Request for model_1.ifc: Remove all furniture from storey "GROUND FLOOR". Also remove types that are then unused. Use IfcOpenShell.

First a look at what the model holds.

```python
import ifcopenshell
import ifcopenshell.util.element

model = ifcopenshell.open("model_1.ifc")
print(model.schema)
storey = next(s for s in model.by_type("IfcBuildingStorey") if s.Name == "GROUND FLOOR")
furniture = [e for e in ifcopenshell.util.element.get_decomposition(storey) if e.is_a("IfcFurnishingElement")]
seen = {}
for e in furniture:
    element_type = ifcopenshell.util.element.get_type(e)
    name = element_type.Name if element_type not in (None, e) else None
    seen[name] = seen.get(name, 0) + 1
for name, count in sorted(seen.items(), key=str):
    print(count, "x", name)
```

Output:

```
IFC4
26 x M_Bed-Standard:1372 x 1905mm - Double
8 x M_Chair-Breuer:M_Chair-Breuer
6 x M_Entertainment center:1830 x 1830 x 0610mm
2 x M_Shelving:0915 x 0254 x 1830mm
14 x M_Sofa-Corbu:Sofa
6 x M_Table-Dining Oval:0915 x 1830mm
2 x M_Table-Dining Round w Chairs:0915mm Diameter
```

```python
import ifcopenshell
import ifcopenshell.api.root
import ifcopenshell.util.element

model = ifcopenshell.open("model_1.ifc")

storey = next(s for s in model.by_type("IfcBuildingStorey") if s.Name == "GROUND FLOOR")
furniture = [e for e in ifcopenshell.util.element.get_decomposition(storey) if e.is_a("IfcFurnishingElement")]
types = {ifcopenshell.util.element.get_type(e) for e in furniture} - {None, *furniture}

for e in furniture:
    ifcopenshell.api.root.remove_product(model, product=e)
print(len(furniture), "removed")

unused = [t for t in types if not ifcopenshell.util.element.get_types(t)]
for t in unused:
    ifcopenshell.api.root.remove_product(model, product=t)
print(len(unused), "unused types removed")

model.write("model_1_v2.ifc")
```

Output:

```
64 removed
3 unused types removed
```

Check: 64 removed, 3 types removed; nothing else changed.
